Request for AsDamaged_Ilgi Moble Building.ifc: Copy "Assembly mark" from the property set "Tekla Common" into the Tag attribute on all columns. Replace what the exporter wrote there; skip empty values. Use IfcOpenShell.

First a look at what the model holds.

```python
import ifcopenshell
import ifcopenshell.util.element

model = ifcopenshell.open("AsDamaged_Ilgi Moble Building.ifc")
print(model.schema)
columns = model.by_type("IfcColumn")
print(len(columns), "columns")
for e in columns[:8]:
    source = ifcopenshell.util.element.get_pset(e, "Tekla Common", "Assembly mark")
    target = e.Tag
    print(e.id(), repr(source), repr(target), sep=" | ")
```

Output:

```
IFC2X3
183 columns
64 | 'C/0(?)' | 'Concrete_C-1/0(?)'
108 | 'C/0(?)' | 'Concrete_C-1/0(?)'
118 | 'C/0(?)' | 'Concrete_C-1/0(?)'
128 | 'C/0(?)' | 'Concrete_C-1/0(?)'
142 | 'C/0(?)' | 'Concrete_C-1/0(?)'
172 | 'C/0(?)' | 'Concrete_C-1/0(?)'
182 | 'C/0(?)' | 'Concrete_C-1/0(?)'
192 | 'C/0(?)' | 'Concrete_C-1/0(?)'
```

```python
import ifcopenshell
import ifcopenshell.util.element

model = ifcopenshell.open("AsDamaged_Ilgi Moble Building.ifc")

count = 0
for e in model.by_type("IfcColumn"):
    value = ifcopenshell.util.element.get_pset(e, "Tekla Common", "Assembly mark")
    current = e.Tag
    if not value or not value.strip() or current == value:
        continue
    e.Tag = value
    count += 1

print(count, "columns updated")

model.write("AsDamaged_Ilgi Moble Building_edited.ifc")
```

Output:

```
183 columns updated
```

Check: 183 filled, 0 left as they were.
